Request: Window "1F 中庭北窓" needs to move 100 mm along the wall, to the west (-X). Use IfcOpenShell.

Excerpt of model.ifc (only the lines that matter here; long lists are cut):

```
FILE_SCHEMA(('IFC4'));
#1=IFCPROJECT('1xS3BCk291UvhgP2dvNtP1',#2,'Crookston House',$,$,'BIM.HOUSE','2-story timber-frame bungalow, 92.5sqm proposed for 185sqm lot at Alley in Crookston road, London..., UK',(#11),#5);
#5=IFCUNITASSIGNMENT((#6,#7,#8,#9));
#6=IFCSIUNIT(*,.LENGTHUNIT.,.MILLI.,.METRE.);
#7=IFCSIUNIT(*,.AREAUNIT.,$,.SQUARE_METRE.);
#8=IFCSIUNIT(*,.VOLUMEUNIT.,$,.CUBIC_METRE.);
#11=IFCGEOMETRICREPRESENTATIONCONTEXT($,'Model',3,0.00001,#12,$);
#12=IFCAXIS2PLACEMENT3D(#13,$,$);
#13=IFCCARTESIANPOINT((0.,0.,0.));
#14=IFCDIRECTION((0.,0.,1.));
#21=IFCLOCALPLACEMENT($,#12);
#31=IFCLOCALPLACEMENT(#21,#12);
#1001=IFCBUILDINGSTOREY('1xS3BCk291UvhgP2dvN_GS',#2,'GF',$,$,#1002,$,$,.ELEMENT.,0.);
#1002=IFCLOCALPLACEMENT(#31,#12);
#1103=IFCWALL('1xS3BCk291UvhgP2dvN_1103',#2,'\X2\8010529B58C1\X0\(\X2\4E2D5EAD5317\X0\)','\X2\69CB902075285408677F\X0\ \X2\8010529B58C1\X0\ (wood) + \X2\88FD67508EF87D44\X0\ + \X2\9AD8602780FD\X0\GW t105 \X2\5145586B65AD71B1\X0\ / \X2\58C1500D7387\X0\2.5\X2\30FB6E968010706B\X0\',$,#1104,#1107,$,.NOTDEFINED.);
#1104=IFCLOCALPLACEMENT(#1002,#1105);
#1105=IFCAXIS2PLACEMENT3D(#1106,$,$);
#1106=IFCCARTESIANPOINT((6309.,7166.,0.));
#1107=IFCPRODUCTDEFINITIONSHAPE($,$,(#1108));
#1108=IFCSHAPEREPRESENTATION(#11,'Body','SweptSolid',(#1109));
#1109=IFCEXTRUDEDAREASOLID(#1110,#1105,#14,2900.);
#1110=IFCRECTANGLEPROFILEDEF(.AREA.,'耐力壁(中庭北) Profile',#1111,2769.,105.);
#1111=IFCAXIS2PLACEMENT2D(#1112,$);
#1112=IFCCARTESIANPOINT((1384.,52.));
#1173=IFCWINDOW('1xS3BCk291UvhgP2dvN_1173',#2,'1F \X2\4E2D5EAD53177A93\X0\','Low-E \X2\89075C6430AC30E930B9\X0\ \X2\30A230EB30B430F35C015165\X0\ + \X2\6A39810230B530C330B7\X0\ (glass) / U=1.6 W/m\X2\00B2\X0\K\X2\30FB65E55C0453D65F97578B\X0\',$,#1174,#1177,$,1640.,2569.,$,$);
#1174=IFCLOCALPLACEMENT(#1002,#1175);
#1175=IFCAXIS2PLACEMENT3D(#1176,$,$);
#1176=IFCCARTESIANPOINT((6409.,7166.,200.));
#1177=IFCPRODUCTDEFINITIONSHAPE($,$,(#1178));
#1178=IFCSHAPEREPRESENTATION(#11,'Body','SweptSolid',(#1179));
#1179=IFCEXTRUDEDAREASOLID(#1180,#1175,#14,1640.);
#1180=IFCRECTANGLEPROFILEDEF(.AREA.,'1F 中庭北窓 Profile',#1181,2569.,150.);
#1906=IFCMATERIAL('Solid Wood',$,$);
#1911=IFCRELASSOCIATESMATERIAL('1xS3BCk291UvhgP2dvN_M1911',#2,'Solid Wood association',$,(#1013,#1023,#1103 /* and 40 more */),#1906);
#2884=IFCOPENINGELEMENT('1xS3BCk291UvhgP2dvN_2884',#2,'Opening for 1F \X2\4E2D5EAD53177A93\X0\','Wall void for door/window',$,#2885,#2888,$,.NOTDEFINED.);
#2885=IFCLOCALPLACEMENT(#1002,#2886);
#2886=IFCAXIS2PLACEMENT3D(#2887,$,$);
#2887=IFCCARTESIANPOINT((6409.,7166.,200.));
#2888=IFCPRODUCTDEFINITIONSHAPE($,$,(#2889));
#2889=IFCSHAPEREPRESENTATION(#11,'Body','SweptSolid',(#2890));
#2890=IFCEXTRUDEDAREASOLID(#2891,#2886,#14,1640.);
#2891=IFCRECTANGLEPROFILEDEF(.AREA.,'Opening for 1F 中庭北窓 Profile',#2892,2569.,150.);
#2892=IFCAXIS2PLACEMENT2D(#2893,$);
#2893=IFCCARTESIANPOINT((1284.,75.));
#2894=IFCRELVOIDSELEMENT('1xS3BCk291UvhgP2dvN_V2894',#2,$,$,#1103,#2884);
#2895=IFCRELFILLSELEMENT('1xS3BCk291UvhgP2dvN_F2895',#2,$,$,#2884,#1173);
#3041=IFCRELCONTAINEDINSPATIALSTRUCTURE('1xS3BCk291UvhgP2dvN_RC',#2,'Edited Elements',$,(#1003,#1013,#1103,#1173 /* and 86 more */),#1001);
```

```python
import ifcopenshell
import ifcopenshell.api.geometry
import ifcopenshell.util.placement

model = ifcopenshell.open("model.ifc")

window = model.by_guid("1xS3BCk291UvhgP2dvN_1173")
opening = window.FillsVoids[0].RelatingOpeningElement
wall = opening.VoidsElements[0].RelatingBuildingElement

wall_matrix = ifcopenshell.util.placement.get_local_placement(wall.ObjectPlacement)
shift = wall_matrix[:3, 0] * -100.0
before = ifcopenshell.util.placement.get_local_placement(window.ObjectPlacement)[:3, 3].copy()

# The window is not placed relative to its opening, so move both.
for product in (opening, window):
    matrix = ifcopenshell.util.placement.get_local_placement(product.ObjectPlacement)
    matrix[:3, 3] += shift
    ifcopenshell.api.geometry.edit_object_placement(model, product=product, matrix=matrix, is_si=False)

after = ifcopenshell.util.placement.get_local_placement(window.ObjectPlacement)[:3, 3]
print("window moved by", (after - before).round(3) + 0.0)

model.write("model_rev.ifc")
```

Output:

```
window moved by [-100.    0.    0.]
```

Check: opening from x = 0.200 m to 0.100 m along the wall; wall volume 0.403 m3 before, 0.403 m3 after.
